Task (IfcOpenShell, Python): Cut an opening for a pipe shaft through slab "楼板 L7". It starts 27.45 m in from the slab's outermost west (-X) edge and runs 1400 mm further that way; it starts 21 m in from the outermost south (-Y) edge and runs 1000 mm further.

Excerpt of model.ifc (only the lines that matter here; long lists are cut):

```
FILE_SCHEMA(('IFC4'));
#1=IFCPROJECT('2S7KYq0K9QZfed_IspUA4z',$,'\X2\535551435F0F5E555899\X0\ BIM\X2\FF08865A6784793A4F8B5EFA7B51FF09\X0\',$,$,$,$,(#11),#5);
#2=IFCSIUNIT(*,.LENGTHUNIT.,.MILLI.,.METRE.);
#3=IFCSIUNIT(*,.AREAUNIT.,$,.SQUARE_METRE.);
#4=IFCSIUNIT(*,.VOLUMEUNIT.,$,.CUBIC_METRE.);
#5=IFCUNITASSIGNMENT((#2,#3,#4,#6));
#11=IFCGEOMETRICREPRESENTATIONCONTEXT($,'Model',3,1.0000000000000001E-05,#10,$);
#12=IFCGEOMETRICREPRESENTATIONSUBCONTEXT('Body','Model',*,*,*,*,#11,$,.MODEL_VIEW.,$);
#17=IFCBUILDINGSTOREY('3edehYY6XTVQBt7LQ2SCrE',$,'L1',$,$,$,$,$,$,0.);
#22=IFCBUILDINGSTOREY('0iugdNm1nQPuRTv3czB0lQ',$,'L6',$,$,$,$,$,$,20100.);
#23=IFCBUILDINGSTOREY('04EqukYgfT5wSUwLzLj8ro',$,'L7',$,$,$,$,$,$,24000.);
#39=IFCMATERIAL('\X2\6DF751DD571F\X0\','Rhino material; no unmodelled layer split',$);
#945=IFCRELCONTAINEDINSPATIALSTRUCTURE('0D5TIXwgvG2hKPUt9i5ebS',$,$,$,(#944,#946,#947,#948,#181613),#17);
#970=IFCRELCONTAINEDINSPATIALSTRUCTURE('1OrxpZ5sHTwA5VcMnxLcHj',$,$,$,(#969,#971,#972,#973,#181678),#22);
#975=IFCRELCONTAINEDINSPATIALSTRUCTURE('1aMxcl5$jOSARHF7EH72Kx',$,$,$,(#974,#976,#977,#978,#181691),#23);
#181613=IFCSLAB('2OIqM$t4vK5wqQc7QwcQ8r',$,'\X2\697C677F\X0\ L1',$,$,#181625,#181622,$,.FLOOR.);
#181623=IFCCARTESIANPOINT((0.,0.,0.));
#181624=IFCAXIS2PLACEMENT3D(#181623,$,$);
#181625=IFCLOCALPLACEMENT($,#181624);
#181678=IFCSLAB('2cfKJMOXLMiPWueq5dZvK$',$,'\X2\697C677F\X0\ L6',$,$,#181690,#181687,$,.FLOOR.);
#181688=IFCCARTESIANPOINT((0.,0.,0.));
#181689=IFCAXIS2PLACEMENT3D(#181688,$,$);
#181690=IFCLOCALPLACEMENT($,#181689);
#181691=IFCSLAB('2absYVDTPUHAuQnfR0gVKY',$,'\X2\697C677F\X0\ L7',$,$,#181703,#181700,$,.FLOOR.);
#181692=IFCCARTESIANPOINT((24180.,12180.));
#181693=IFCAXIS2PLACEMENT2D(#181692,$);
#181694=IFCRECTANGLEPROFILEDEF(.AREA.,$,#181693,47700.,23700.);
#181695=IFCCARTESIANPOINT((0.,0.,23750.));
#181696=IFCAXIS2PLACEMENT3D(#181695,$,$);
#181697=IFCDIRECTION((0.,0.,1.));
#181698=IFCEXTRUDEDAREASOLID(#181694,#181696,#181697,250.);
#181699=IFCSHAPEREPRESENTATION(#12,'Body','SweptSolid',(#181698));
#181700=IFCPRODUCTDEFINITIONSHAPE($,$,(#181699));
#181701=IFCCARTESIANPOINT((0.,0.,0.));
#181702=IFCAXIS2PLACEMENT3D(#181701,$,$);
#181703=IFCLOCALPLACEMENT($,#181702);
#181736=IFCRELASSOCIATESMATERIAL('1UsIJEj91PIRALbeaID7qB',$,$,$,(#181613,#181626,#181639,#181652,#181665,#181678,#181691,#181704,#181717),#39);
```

```python
import numpy as np
import ifcopenshell
import ifcopenshell.api.feature
import ifcopenshell.api.geometry
import ifcopenshell.api.root
import ifcopenshell.geom
import ifcopenshell.util.placement
import ifcopenshell.util.representation
import ifcopenshell.util.shape
import ifcopenshell.util.unit

model = ifcopenshell.open("model.ifc")
unit_scale = ifcopenshell.util.unit.calculate_unit_scale(model)
settings = ifcopenshell.geom.settings()


def volume(element):
    """Net volume in cubic metres, openings subtracted."""
    shape = ifcopenshell.geom.create_shape(settings, element)
    return ifcopenshell.util.shape.get_volume(shape.geometry)


slab = model.by_guid("2absYVDTPUHAuQnfR0gVKY")
before = volume(slab)

# Extent in the slab's own axes, in metres. The edges named are its -X and -Y sides.
slab_shape = ifcopenshell.geom.create_shape(settings, slab)
vertices = ifcopenshell.util.shape.get_vertices(slab_shape.geometry)
x_min, y_min, bottom = vertices.min(axis=0)
top = vertices[:, 2].max()

opening = ifcopenshell.api.root.create_entity(model, ifc_class="IfcOpeningElement", name="Pipe shaft opening", predefined_type="OPENING")
context = ifcopenshell.util.representation.get_context(model, "Model", "Body", "MODEL_VIEW")
width, depth = 1.4, 1
outline = [(0.0, 0.0), (width, 0.0), (width, depth), (0.0, depth), (0.0, 0.0)]
# Overshoot both faces by 50 mm so the cut is clean.
shape = ifcopenshell.api.geometry.add_slab_representation(
    model, context=context, depth=top - bottom + 0.1, polyline=outline
)
ifcopenshell.api.geometry.assign_representation(model, product=opening, representation=shape)

matrix = ifcopenshell.util.placement.get_local_placement(slab.ObjectPlacement)
matrix[:, 3] = matrix @ np.append(np.array([x_min + 27.45, y_min + 21, bottom - 0.05]) / unit_scale, 1.0)
ifcopenshell.api.geometry.edit_object_placement(model, product=opening, matrix=matrix, is_si=False)
ifcopenshell.api.feature.add_feature(model, feature=opening, element=slab)

after = volume(slab)

print(f"slab volume {before:.3f} -> {after:.3f} m3")

model.write("model_rev.ifc")
```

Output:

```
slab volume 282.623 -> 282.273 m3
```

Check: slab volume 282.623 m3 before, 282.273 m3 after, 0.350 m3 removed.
